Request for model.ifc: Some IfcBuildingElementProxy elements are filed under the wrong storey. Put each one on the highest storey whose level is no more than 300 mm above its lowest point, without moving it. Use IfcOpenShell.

First a look at what the model holds.

```python
import ifcopenshell
import ifcopenshell.util.element
import ifcopenshell.util.placement

model = ifcopenshell.open("model.ifc")
print(model.schema)
for storey in model.by_type("IfcBuildingStorey"):
    level = ifcopenshell.util.placement.get_storey_elevation(storey)
    count = sum(e.is_a("IfcBuildingElementProxy") for e in ifcopenshell.util.element.get_contained(storey))
    print(storey.id(), storey.Name, round(level, 3), count, sep=" | ")
```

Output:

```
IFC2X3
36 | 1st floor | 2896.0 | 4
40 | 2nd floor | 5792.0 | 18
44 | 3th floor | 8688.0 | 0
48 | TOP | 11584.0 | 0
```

```python
import ifcopenshell
import ifcopenshell.api.spatial
import ifcopenshell.geom
import ifcopenshell.util.element
import ifcopenshell.util.placement
import ifcopenshell.util.shape
import ifcopenshell.util.unit

model = ifcopenshell.open("model.ifc")
unit_scale = ifcopenshell.util.unit.calculate_unit_scale(model)
settings = ifcopenshell.geom.settings()

levels = sorted(
    ((ifcopenshell.util.placement.get_storey_elevation(s) * unit_scale, s) for s in model.by_type("IfcBuildingStorey")),
    key=lambda pair: pair[0],
)

for e in model.by_type("IfcBuildingElementProxy"):
    current = e.ContainedInStructure[0].RelatingStructure if e.ContainedInStructure else None
    if current is None or not current.is_a("IfcBuildingStorey"):
        continue
    shape = ifcopenshell.geom.create_shape(settings, e)
    bottom = ifcopenshell.util.shape.get_shape_bottom_elevation(shape, shape.geometry)
    below = [s for level, s in levels if level <= bottom + 0.3]
    storey = below[-1] if below else levels[0][1]
    if storey != current:
        # assign_container keeps the world position.
        ifcopenshell.api.spatial.assign_container(model, products=[e], relating_structure=storey)
        print(e.id(), current.Name, "->", storey.Name)

model.write("model-out.ifc")
```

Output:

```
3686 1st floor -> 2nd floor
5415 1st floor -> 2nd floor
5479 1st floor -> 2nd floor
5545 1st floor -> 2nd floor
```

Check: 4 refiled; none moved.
